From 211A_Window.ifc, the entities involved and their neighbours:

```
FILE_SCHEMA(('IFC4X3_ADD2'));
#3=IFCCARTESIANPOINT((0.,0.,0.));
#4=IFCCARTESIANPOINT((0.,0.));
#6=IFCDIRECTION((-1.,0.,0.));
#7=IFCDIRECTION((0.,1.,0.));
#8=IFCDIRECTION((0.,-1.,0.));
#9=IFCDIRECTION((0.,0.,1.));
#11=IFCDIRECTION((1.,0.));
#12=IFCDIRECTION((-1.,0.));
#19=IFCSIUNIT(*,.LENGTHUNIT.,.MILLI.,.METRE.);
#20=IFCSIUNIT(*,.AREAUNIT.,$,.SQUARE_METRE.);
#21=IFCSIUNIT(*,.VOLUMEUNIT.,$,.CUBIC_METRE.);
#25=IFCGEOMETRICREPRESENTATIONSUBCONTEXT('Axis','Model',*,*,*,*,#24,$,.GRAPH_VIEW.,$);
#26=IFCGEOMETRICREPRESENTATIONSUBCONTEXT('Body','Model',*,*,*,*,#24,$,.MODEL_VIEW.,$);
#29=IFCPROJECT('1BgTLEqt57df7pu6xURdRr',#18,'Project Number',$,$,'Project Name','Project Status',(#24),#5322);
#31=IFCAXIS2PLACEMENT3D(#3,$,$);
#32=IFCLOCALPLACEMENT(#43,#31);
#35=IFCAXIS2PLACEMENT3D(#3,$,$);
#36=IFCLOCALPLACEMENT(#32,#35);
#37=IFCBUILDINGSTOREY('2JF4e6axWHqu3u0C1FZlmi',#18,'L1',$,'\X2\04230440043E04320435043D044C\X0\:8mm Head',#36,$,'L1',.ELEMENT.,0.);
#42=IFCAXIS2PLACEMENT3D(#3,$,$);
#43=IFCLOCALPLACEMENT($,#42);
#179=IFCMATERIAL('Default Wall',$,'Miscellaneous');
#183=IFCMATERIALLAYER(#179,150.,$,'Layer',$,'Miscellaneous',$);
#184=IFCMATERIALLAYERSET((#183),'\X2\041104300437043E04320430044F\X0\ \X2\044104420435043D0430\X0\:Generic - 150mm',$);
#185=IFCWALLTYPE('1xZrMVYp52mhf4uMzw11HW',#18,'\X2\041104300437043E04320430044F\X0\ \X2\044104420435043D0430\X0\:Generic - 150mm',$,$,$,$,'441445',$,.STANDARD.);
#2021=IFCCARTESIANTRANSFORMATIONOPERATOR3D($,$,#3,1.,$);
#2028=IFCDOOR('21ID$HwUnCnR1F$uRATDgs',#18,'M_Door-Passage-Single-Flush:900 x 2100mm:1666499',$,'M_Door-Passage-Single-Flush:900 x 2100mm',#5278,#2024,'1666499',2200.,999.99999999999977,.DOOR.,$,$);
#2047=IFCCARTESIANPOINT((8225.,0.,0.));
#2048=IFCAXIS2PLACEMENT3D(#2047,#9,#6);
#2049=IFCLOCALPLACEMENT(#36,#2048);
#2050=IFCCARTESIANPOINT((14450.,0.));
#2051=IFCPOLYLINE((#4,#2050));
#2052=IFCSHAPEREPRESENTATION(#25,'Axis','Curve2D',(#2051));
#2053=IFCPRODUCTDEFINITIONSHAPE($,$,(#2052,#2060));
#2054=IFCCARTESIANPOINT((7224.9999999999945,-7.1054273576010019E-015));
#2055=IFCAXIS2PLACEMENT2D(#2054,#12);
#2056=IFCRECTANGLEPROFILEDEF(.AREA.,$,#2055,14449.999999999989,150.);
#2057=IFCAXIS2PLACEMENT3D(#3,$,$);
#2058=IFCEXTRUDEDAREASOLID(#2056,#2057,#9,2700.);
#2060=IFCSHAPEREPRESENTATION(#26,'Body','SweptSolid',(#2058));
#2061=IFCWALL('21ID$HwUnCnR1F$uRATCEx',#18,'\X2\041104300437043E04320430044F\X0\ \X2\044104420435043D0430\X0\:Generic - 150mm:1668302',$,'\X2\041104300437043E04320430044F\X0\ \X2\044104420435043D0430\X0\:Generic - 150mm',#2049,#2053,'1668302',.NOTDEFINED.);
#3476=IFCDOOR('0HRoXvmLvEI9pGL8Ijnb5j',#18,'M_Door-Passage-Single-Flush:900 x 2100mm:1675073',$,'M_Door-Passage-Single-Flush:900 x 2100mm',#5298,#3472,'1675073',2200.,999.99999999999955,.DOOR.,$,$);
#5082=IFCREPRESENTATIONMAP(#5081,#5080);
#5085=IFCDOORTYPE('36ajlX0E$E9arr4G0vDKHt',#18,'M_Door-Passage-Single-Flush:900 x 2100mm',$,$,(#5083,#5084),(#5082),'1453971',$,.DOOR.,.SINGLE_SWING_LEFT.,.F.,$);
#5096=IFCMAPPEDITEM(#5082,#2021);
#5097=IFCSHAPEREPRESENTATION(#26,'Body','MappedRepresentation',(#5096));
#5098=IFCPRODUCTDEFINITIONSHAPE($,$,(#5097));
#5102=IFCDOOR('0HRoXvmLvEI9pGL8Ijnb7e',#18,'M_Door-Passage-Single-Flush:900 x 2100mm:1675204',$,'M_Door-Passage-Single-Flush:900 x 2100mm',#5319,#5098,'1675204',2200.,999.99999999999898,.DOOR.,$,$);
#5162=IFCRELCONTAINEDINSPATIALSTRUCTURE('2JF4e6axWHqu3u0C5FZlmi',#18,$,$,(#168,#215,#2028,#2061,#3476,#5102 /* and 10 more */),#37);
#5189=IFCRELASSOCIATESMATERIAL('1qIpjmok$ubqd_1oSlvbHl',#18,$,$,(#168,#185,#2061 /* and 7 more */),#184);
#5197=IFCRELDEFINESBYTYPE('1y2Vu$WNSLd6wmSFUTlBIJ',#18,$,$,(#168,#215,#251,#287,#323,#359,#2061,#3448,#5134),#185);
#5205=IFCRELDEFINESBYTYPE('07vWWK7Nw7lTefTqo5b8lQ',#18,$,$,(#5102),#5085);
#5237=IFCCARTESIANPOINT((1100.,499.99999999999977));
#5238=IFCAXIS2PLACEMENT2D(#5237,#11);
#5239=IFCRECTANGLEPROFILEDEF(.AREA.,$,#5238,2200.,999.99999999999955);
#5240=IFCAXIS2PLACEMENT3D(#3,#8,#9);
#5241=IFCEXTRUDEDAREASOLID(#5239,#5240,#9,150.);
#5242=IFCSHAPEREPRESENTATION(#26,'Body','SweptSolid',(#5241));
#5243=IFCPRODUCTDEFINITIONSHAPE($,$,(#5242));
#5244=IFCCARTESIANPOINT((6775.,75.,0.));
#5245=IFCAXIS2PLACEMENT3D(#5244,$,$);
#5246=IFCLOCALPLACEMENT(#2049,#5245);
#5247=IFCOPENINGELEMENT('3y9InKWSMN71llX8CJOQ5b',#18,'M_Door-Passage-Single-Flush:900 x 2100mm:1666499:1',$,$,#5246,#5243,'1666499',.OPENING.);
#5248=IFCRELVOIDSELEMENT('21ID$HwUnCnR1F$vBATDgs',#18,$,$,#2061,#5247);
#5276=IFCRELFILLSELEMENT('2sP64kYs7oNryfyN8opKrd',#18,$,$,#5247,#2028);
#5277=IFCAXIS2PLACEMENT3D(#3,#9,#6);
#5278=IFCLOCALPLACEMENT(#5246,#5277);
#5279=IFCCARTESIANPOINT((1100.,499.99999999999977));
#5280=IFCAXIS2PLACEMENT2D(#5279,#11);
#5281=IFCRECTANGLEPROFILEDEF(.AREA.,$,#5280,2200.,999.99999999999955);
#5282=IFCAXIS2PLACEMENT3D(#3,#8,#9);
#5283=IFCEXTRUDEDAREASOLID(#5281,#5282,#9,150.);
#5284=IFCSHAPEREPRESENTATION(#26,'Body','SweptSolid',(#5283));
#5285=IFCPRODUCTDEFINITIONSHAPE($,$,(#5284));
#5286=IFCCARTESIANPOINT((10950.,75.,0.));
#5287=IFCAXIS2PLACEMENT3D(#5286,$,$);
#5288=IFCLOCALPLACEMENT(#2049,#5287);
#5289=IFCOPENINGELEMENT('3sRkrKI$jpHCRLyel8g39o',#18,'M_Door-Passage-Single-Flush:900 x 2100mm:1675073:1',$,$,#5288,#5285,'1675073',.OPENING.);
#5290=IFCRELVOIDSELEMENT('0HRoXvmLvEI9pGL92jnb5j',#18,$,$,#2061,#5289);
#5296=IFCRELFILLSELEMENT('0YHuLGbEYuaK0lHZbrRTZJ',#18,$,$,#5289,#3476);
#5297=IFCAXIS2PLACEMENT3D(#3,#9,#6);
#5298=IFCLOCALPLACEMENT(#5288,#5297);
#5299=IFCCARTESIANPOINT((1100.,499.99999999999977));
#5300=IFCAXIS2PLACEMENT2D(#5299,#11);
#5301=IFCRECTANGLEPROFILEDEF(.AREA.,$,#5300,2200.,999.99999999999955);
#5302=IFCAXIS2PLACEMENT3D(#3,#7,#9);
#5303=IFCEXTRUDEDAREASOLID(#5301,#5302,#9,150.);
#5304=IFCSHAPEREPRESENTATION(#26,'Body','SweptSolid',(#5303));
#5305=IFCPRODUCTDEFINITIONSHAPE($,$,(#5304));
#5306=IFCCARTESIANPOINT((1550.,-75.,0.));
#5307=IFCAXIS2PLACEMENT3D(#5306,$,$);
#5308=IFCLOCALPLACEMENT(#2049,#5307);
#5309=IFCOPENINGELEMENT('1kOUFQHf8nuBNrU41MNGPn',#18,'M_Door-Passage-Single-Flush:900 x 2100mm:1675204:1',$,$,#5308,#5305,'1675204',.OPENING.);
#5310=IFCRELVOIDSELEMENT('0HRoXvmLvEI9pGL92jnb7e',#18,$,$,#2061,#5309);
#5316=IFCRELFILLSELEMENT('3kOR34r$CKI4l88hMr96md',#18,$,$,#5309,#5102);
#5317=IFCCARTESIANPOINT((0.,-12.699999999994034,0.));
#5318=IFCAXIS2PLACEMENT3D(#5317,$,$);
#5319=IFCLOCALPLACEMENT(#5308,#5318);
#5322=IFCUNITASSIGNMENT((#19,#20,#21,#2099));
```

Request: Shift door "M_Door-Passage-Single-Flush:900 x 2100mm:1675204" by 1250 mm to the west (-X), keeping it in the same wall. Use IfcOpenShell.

```python
import ifcopenshell
import ifcopenshell.api.geometry
import ifcopenshell.util.placement
import ifcopenshell.util.unit

model = ifcopenshell.open("211A_Window.ifc")
unit_scale = ifcopenshell.util.unit.calculate_unit_scale(model)

door = model.by_guid("0HRoXvmLvEI9pGL8Ijnb7e")
opening = door.FillsVoids[0].RelatingOpeningElement
wall = opening.VoidsElements[0].RelatingBuildingElement

wall_matrix = ifcopenshell.util.placement.get_local_placement(wall.ObjectPlacement)
shift = wall_matrix[:3, 0] * 1.25 / unit_scale
before = ifcopenshell.util.placement.get_local_placement(door.ObjectPlacement)[:3, 3].copy()

# The door is placed relative to its opening, so it follows when the opening moves.
matrix = ifcopenshell.util.placement.get_local_placement(opening.ObjectPlacement)
matrix[:3, 3] += shift
ifcopenshell.api.geometry.edit_object_placement(
    model, product=opening, matrix=matrix, is_si=False, should_transform_children=True
)

after = ifcopenshell.util.placement.get_local_placement(door.ObjectPlacement)[:3, 3]
print("door moved by", (after - before).round(3) + 0.0)

model.write("211A_Window_rev.ifc")
```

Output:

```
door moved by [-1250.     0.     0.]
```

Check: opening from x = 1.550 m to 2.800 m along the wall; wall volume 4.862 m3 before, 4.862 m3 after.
